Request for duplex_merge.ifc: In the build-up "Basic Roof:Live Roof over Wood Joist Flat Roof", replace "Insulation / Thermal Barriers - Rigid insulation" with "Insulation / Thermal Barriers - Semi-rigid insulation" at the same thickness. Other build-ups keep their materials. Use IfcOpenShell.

First a look at what the model holds.

```python
import ifcopenshell
import ifcopenshell.util.element

model = ifcopenshell.open("duplex_merge.ifc")
print(model.schema)
for layer_set in model.by_type("IfcMaterialLayerSet"):
    if layer_set.LayerSetName == "Basic Roof:Live Roof over Wood Joist Flat Roof":
        for layer in layer_set.MaterialLayers:
            print(layer.id(), layer.Material and layer.Material.Name, layer.LayerThickness, sep=" | ")
        print(len(ifcopenshell.util.element.get_elements_by_material(model, layer_set)), "elements and types use it")
print(sorted(m.Name for m in model.by_type("IfcMaterial") if m.Name)[:60])
```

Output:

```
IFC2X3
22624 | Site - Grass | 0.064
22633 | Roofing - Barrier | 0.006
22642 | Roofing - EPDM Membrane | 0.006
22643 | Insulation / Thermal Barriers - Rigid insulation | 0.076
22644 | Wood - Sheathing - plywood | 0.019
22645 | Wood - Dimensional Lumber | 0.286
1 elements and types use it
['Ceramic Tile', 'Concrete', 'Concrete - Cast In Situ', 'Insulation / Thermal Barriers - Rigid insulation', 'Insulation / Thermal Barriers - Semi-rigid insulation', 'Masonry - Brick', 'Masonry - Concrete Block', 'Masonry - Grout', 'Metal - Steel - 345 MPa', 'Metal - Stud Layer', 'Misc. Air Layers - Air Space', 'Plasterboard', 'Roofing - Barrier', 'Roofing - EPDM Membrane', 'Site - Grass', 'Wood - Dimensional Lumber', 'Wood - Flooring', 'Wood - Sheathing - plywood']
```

```python
import ifcopenshell
import ifcopenshell.api.material

model = ifcopenshell.open("duplex_merge.ifc")

layer_set = next(s for s in model.by_type("IfcMaterialLayerSet") if s.LayerSetName == "Basic Roof:Live Roof over Wood Joist Flat Roof")
layer = next(l for l in layer_set.MaterialLayers if l.Material and l.Material.Name == "Insulation / Thermal Barriers - Rigid insulation")
material = next(m for m in model.by_type("IfcMaterial") if m.Name == "Insulation / Thermal Barriers - Semi-rigid insulation")

# Point this one layer at the other material; renaming the old one would change it everywhere.
ifcopenshell.api.material.edit_layer(model, layer=layer, attributes={}, material=material)

print([l.Material.Name if l.Material else None for l in layer_set.MaterialLayers])

model.write("duplex_merge_updated.ifc")
```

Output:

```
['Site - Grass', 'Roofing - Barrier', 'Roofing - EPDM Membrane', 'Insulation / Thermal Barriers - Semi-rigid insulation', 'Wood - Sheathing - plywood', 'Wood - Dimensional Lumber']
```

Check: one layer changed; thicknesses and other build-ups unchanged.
